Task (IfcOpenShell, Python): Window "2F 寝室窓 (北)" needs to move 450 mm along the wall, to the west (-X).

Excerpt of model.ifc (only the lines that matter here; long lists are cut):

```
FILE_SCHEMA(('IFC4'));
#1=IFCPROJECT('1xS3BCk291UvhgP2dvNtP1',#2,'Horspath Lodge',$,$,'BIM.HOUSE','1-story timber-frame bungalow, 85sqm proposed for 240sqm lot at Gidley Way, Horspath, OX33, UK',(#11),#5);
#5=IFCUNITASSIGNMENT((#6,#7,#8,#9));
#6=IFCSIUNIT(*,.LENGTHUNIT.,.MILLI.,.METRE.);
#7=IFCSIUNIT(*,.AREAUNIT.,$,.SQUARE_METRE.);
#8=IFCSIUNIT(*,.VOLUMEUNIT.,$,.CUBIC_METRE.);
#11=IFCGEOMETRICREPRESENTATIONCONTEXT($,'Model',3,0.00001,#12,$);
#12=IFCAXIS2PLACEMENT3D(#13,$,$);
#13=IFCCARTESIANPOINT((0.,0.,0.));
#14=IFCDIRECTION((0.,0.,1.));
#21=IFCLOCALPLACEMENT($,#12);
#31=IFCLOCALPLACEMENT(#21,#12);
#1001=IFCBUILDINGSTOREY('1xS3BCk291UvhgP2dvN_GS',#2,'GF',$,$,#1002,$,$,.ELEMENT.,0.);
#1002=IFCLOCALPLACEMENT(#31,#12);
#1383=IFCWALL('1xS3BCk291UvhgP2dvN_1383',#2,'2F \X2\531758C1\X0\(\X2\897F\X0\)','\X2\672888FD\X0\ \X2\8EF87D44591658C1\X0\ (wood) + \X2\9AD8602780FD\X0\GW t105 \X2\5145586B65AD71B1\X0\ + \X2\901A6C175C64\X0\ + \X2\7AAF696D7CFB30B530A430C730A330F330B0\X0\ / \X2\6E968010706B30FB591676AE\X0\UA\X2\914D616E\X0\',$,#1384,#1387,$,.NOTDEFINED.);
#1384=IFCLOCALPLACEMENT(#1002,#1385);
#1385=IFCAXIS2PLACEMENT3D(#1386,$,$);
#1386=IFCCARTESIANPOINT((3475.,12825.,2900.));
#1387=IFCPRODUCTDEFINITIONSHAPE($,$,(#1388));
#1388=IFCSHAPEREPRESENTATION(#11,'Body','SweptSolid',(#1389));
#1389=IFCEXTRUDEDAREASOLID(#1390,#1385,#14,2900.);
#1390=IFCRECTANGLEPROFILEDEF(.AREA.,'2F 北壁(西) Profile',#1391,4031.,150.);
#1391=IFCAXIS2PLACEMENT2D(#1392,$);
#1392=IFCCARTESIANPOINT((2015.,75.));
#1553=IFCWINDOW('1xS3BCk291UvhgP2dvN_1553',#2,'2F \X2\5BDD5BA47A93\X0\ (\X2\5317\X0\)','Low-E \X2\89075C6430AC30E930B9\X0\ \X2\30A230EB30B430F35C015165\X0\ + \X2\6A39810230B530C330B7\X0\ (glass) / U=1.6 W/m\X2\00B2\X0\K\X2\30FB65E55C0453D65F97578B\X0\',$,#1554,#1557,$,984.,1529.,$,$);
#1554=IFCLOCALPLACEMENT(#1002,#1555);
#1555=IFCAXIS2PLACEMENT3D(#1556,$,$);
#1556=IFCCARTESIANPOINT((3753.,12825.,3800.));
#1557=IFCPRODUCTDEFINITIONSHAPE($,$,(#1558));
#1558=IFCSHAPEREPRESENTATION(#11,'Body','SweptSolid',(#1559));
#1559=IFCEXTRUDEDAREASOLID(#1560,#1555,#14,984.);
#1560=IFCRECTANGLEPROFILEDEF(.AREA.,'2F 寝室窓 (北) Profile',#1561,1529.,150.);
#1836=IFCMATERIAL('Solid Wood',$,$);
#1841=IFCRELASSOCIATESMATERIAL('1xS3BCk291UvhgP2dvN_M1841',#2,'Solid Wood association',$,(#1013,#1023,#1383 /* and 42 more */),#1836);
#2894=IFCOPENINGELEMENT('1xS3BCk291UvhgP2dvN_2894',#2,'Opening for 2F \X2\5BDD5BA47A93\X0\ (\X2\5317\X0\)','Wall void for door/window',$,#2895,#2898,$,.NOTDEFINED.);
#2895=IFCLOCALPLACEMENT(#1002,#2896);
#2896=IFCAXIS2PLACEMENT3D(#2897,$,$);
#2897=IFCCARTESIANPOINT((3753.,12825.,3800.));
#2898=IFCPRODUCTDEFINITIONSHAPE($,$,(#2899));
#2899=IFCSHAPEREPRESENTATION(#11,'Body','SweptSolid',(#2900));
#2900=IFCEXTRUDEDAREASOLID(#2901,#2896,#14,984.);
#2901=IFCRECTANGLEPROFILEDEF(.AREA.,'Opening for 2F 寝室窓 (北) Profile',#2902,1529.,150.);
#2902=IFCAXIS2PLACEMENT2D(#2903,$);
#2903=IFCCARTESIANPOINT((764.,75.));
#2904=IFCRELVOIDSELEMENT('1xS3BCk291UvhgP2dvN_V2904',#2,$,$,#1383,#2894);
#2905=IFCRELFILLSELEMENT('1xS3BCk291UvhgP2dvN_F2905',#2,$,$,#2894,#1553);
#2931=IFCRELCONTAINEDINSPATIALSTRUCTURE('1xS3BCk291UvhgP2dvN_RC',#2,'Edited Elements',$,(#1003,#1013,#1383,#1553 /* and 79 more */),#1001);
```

```python
import ifcopenshell
import ifcopenshell.api.geometry
import ifcopenshell.util.placement
import ifcopenshell.util.unit

model = ifcopenshell.open("model.ifc")
unit_scale = ifcopenshell.util.unit.calculate_unit_scale(model)

window = model.by_id(1553)
opening = window.FillsVoids[0].RelatingOpeningElement
wall = opening.VoidsElements[0].RelatingBuildingElement

wall_matrix = ifcopenshell.util.placement.get_local_placement(wall.ObjectPlacement)
shift = wall_matrix[:3, 0] * -0.45 / unit_scale
before = ifcopenshell.util.placement.get_local_placement(window.ObjectPlacement)[:3, 3].copy()

# The window is not placed relative to its opening, so move both.
for product in (opening, window):
    matrix = ifcopenshell.util.placement.get_local_placement(product.ObjectPlacement)
    matrix[:3, 3] += shift
    ifcopenshell.api.geometry.edit_object_placement(model, product=product, matrix=matrix, is_si=False)

after = ifcopenshell.util.placement.get_local_placement(window.ObjectPlacement)[:3, 3]
print("window moved by", (after - before).round(3) + 0.0)

model.write("model-out.ifc")
```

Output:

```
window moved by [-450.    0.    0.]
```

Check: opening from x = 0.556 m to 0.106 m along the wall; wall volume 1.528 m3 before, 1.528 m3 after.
